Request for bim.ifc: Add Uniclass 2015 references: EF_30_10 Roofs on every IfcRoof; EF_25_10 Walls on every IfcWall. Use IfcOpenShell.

First a look at what the model holds.

```python
import ifcopenshell

model = ifcopenshell.open("bim.ifc")
print(model.schema)
print("classifications:", [c.Name for c in model.by_type("IfcClassification")])
for ifc_class in ("IfcDoor", "IfcRoof", "IfcStair", "IfcWall", "IfcWindow"):
    print(ifc_class, len(model.by_type(ifc_class)))
```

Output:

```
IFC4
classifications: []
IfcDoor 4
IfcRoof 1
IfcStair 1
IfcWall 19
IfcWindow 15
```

```python
import ifcopenshell
import ifcopenshell.api.classification

model = ifcopenshell.open("bim.ifc")

system = ifcopenshell.api.classification.add_classification(model, classification="Uniclass 2015")

codes = {
    "IfcRoof": ("EF_30_10", "Roofs"),
    "IfcWall": ("EF_25_10", "Walls"),
}
for ifc_class, (code, name) in codes.items():
    products = model.by_type(ifc_class)
    ifcopenshell.api.classification.add_reference(
        model, products=products, classification=system, identification=code, name=name
    )
    print(code, len(products))

model.write("bim_rev.ifc")
```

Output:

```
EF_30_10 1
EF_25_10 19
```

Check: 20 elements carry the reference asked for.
